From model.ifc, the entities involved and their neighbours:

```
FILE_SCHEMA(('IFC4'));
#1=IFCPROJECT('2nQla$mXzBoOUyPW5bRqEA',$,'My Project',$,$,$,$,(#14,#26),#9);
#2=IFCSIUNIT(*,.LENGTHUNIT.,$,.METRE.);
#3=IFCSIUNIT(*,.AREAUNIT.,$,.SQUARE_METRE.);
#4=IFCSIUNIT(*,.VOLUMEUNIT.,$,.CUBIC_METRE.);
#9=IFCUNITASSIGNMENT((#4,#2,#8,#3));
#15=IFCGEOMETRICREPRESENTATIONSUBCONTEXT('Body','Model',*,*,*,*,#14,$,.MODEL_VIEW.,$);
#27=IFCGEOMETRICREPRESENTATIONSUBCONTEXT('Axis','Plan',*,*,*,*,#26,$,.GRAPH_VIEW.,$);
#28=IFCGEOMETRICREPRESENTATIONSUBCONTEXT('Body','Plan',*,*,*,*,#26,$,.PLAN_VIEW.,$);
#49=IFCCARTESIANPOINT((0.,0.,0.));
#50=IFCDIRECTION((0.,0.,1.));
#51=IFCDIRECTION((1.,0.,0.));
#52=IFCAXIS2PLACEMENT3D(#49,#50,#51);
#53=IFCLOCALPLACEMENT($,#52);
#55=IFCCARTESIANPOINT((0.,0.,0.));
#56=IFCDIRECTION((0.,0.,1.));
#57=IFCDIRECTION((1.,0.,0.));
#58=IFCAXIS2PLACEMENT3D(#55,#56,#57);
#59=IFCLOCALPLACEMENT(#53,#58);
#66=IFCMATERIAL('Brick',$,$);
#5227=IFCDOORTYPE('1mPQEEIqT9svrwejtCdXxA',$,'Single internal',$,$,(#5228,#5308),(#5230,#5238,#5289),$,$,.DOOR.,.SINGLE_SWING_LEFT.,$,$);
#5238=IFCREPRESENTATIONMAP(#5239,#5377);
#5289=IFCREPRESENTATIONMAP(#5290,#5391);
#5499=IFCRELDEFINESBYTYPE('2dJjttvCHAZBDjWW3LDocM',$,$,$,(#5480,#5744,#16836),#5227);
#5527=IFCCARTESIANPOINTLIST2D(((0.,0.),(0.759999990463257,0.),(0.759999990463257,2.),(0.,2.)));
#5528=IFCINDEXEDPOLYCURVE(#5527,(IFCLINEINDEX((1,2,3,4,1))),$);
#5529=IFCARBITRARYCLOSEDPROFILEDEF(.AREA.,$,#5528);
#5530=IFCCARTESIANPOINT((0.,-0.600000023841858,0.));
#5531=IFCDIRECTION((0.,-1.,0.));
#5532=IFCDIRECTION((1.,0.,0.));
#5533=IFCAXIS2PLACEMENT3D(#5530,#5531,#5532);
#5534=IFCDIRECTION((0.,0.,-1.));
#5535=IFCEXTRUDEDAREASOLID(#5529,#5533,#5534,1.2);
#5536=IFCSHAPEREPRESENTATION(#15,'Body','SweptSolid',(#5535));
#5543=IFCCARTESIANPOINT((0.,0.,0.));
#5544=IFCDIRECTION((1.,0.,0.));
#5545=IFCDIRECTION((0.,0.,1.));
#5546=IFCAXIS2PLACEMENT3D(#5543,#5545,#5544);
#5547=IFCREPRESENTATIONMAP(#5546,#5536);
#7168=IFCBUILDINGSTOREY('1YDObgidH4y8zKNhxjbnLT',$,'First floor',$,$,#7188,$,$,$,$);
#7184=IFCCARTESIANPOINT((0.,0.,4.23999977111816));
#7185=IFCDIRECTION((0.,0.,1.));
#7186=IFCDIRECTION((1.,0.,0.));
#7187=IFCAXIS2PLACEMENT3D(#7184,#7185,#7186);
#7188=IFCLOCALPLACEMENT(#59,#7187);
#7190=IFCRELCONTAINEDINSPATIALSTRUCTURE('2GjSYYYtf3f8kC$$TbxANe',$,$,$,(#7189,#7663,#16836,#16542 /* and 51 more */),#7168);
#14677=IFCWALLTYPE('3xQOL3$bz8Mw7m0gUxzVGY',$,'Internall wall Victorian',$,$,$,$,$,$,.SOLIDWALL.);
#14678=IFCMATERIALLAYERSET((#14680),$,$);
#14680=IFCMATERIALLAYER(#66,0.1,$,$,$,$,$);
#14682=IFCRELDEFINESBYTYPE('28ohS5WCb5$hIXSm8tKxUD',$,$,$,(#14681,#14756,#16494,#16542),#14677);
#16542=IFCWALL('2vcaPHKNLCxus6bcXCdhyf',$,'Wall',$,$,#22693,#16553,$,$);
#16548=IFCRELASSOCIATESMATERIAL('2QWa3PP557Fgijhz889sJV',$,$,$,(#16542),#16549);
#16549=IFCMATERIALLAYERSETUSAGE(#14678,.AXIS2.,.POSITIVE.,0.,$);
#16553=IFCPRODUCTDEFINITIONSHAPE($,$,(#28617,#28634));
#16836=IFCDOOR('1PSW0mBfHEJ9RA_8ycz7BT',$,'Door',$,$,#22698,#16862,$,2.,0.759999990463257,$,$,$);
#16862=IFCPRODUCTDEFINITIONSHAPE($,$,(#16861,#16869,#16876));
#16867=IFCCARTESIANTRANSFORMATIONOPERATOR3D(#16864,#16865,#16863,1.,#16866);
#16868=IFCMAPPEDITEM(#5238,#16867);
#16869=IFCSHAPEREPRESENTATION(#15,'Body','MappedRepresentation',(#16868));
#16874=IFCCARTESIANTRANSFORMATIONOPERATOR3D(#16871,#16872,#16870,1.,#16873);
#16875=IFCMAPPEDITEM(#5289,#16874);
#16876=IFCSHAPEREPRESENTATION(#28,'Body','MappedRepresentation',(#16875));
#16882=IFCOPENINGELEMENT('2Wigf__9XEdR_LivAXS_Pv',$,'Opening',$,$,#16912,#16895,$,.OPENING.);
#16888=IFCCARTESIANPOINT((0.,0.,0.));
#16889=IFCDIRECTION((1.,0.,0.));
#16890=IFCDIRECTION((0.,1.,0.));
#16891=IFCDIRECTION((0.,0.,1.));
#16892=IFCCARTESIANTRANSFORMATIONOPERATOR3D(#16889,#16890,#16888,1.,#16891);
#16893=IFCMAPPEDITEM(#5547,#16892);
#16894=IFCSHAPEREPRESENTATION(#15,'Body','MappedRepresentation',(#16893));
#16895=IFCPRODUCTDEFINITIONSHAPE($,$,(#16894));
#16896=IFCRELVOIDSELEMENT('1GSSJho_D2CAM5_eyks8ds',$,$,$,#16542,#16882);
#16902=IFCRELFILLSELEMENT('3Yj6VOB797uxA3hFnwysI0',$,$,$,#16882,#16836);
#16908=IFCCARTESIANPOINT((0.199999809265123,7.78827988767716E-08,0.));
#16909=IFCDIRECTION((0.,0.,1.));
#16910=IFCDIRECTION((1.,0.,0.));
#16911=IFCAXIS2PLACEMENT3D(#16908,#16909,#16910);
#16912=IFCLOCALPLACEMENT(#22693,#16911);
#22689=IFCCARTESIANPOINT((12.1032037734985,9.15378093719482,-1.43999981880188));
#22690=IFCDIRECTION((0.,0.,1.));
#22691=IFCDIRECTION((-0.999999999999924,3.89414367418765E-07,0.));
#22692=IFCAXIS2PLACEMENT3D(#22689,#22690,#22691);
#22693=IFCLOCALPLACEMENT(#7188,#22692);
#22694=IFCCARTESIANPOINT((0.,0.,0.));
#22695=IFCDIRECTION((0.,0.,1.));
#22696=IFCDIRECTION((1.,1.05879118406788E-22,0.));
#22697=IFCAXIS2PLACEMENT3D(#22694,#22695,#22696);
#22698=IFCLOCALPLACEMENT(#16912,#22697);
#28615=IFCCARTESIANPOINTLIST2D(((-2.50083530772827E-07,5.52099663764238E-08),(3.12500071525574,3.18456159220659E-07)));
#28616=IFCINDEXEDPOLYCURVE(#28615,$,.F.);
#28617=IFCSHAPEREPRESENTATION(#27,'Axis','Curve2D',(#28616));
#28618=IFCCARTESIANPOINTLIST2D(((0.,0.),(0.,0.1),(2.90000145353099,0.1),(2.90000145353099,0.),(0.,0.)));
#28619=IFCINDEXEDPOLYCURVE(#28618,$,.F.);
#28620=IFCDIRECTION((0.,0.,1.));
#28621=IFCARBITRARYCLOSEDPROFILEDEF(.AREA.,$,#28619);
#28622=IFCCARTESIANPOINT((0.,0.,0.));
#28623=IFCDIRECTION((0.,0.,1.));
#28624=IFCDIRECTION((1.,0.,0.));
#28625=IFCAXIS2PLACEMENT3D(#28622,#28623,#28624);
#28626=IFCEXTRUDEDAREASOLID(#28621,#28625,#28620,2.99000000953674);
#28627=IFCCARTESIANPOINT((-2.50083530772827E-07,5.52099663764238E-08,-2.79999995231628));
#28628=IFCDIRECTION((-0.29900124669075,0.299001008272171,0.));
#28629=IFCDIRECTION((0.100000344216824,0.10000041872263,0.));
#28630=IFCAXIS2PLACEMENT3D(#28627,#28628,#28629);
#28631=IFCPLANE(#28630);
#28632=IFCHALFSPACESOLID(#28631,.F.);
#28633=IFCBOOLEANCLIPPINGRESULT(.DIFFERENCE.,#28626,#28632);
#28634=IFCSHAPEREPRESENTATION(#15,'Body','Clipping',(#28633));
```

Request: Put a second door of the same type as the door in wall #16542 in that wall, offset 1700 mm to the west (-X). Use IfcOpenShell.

```python
import ifcopenshell
import ifcopenshell.api.feature
import ifcopenshell.api.geometry
import ifcopenshell.api.root
import ifcopenshell.geom
import ifcopenshell.util.element
import ifcopenshell.util.placement
import ifcopenshell.util.shape

model = ifcopenshell.open("model.ifc")
settings = ifcopenshell.geom.settings()


def volume(element):
    """Net volume in cubic metres, openings subtracted."""
    shape = ifcopenshell.geom.create_shape(settings, element)
    return ifcopenshell.util.shape.get_volume(shape.geometry)


door = model.by_id(16836)
opening = door.FillsVoids[0].RelatingOpeningElement
wall = opening.VoidsElements[0].RelatingBuildingElement
before = volume(wall)
shift = ifcopenshell.util.placement.get_local_placement(wall.ObjectPlacement)[:3, 0] * 1.7

# copy_class copies the void relationship, type, container and properties, but no geometry.
new_opening = ifcopenshell.api.root.copy_class(model, product=opening)
new_opening.Representation = ifcopenshell.util.element.copy_deep(
    model, opening.Representation, exclude=["IfcGeometricRepresentationContext", "IfcRepresentationMap"]
)
new_door = ifcopenshell.api.root.copy_class(model, product=door)
new_door.Representation = ifcopenshell.util.element.copy_deep(
    model, door.Representation, exclude=["IfcGeometricRepresentationContext", "IfcRepresentationMap"]
)
ifcopenshell.api.feature.add_filling(model, opening=new_opening, element=new_door)

for old, new in ((opening, new_opening), (door, new_door)):
    matrix = ifcopenshell.util.placement.get_local_placement(old.ObjectPlacement)
    matrix[:3, 3] += shift
    ifcopenshell.api.geometry.edit_object_placement(model, product=new, matrix=matrix, is_si=False)

after = volume(wall)

print(f"wall volume {before:.3f} -> {after:.3f} m3")

model.write("model_rev.ifc")
```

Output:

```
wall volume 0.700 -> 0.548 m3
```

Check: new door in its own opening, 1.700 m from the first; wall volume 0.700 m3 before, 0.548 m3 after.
